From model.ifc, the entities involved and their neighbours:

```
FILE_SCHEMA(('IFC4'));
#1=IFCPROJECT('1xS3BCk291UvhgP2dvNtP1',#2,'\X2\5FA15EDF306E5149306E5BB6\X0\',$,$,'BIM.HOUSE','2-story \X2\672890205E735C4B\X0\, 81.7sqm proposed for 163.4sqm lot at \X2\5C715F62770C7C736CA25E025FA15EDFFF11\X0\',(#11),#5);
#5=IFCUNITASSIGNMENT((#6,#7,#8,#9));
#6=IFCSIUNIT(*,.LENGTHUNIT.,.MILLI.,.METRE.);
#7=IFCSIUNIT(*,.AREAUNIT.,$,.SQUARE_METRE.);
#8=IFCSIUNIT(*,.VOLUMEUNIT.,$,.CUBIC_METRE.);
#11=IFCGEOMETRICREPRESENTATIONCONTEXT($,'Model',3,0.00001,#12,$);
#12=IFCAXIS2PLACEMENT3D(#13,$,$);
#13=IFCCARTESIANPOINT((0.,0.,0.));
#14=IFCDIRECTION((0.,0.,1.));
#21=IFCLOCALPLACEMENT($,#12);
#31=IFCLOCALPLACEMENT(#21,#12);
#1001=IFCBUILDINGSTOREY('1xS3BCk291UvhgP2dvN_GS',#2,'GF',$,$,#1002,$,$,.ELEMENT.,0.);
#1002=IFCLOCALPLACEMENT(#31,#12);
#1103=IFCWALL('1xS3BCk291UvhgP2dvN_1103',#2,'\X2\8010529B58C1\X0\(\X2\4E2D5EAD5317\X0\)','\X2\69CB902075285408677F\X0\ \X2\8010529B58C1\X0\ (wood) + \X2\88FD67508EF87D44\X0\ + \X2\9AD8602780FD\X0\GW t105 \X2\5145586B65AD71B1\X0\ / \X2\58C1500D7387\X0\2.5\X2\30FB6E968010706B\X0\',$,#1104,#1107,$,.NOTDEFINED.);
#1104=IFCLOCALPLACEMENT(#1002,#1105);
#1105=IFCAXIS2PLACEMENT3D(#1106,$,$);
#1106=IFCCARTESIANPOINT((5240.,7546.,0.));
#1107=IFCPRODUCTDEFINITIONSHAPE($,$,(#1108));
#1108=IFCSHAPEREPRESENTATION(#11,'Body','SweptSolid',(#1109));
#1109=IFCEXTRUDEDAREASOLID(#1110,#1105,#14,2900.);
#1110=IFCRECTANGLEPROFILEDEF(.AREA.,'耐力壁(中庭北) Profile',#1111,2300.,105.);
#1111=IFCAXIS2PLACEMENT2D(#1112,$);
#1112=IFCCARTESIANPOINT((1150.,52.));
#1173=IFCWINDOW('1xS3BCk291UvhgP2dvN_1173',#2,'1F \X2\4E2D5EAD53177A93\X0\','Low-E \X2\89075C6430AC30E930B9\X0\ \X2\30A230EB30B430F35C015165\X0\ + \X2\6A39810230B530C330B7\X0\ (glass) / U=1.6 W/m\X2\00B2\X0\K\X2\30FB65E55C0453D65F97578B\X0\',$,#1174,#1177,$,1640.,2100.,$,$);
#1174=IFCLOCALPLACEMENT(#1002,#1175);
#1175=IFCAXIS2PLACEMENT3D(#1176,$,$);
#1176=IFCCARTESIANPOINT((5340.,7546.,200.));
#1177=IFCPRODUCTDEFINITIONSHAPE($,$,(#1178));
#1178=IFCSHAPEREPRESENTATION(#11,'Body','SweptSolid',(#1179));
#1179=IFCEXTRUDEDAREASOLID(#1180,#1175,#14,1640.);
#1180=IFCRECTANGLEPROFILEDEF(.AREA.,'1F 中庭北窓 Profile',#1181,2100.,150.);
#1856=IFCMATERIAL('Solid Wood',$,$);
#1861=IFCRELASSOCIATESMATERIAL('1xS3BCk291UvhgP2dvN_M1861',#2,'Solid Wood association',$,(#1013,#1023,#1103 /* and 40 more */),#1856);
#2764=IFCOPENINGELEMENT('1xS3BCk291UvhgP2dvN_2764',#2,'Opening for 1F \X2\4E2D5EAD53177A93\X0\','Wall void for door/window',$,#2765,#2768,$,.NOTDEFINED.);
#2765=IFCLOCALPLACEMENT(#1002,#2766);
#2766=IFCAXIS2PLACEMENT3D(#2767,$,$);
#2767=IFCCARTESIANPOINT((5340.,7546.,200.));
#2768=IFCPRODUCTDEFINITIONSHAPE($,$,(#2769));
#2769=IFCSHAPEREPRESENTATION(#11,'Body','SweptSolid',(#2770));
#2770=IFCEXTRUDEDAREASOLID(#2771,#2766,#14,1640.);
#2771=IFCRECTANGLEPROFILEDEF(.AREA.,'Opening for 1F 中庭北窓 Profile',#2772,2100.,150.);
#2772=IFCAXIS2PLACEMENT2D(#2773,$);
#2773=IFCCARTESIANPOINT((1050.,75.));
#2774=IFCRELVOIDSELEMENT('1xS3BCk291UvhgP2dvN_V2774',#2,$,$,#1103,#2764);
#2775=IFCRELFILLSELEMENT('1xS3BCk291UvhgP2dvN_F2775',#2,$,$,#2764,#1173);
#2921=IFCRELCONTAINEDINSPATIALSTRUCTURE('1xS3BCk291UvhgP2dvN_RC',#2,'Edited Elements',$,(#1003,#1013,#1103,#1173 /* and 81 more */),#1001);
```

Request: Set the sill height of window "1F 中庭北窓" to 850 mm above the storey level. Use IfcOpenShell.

```python
import numpy as np
import ifcopenshell
import ifcopenshell.api.geometry
import ifcopenshell.geom
import ifcopenshell.util.element
import ifcopenshell.util.placement
import ifcopenshell.util.shape
import ifcopenshell.util.unit

model = ifcopenshell.open("model.ifc")
unit_scale = ifcopenshell.util.unit.calculate_unit_scale(model)

window = model.by_guid("1xS3BCk291UvhgP2dvN_1173")
opening = window.FillsVoids[0].RelatingOpeningElement
storey = ifcopenshell.util.element.get_container(window, ifc_class="IfcBuildingStorey")
level = ifcopenshell.util.placement.get_local_placement(storey.ObjectPlacement)[2, 3]

# The opening's origin need not be at the sill, so measure its lowest point.
shape = ifcopenshell.geom.create_shape(ifcopenshell.geom.settings(), opening)
bottom = ifcopenshell.util.shape.get_shape_bottom_elevation(shape, shape.geometry) / unit_scale
dz = level + 850.0 - bottom

shift = np.array([0.0, 0.0, dz])
# The window is not placed relative to its opening, so move both.
for product in (opening, window):
    matrix = ifcopenshell.util.placement.get_local_placement(product.ObjectPlacement)
    matrix[:3, 3] += shift
    ifcopenshell.api.geometry.edit_object_placement(model, product=product, matrix=matrix, is_si=False)

print(f"moved by {dz * unit_scale:+.3f} m")

model.write("model_edited.ifc")
```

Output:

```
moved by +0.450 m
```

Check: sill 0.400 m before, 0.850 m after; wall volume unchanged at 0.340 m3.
